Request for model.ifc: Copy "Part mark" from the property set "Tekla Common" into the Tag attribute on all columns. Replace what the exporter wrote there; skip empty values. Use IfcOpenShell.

First a look at what the model holds.

```python
import ifcopenshell
import ifcopenshell.util.element

model = ifcopenshell.open("model.ifc")
print(model.schema)
columns = model.by_type("IfcColumn")
print(len(columns), "columns")
for e in columns[:8]:
    source = ifcopenshell.util.element.get_pset(e, "Tekla Common", "Part mark")
    target = e.Tag
    print(e.id(), repr(source), repr(target), sep=" | ")
```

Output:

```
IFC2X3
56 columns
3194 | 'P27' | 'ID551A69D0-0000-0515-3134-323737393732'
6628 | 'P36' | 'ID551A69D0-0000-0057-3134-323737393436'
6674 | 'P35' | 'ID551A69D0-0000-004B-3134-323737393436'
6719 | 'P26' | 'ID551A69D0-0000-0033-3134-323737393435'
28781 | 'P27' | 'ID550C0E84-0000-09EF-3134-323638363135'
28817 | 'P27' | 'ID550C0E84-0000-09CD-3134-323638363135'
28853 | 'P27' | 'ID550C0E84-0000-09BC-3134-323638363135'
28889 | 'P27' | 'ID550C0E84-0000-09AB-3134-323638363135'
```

```python
import ifcopenshell
import ifcopenshell.util.element

model = ifcopenshell.open("model.ifc")

count = 0
for e in model.by_type("IfcColumn"):
    value = ifcopenshell.util.element.get_pset(e, "Tekla Common", "Part mark")
    current = e.Tag
    if not value or not value.strip() or current == value:
        continue
    e.Tag = value
    count += 1

print(count, "columns updated")

model.write("model_v2.ifc")
```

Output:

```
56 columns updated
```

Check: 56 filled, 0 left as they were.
